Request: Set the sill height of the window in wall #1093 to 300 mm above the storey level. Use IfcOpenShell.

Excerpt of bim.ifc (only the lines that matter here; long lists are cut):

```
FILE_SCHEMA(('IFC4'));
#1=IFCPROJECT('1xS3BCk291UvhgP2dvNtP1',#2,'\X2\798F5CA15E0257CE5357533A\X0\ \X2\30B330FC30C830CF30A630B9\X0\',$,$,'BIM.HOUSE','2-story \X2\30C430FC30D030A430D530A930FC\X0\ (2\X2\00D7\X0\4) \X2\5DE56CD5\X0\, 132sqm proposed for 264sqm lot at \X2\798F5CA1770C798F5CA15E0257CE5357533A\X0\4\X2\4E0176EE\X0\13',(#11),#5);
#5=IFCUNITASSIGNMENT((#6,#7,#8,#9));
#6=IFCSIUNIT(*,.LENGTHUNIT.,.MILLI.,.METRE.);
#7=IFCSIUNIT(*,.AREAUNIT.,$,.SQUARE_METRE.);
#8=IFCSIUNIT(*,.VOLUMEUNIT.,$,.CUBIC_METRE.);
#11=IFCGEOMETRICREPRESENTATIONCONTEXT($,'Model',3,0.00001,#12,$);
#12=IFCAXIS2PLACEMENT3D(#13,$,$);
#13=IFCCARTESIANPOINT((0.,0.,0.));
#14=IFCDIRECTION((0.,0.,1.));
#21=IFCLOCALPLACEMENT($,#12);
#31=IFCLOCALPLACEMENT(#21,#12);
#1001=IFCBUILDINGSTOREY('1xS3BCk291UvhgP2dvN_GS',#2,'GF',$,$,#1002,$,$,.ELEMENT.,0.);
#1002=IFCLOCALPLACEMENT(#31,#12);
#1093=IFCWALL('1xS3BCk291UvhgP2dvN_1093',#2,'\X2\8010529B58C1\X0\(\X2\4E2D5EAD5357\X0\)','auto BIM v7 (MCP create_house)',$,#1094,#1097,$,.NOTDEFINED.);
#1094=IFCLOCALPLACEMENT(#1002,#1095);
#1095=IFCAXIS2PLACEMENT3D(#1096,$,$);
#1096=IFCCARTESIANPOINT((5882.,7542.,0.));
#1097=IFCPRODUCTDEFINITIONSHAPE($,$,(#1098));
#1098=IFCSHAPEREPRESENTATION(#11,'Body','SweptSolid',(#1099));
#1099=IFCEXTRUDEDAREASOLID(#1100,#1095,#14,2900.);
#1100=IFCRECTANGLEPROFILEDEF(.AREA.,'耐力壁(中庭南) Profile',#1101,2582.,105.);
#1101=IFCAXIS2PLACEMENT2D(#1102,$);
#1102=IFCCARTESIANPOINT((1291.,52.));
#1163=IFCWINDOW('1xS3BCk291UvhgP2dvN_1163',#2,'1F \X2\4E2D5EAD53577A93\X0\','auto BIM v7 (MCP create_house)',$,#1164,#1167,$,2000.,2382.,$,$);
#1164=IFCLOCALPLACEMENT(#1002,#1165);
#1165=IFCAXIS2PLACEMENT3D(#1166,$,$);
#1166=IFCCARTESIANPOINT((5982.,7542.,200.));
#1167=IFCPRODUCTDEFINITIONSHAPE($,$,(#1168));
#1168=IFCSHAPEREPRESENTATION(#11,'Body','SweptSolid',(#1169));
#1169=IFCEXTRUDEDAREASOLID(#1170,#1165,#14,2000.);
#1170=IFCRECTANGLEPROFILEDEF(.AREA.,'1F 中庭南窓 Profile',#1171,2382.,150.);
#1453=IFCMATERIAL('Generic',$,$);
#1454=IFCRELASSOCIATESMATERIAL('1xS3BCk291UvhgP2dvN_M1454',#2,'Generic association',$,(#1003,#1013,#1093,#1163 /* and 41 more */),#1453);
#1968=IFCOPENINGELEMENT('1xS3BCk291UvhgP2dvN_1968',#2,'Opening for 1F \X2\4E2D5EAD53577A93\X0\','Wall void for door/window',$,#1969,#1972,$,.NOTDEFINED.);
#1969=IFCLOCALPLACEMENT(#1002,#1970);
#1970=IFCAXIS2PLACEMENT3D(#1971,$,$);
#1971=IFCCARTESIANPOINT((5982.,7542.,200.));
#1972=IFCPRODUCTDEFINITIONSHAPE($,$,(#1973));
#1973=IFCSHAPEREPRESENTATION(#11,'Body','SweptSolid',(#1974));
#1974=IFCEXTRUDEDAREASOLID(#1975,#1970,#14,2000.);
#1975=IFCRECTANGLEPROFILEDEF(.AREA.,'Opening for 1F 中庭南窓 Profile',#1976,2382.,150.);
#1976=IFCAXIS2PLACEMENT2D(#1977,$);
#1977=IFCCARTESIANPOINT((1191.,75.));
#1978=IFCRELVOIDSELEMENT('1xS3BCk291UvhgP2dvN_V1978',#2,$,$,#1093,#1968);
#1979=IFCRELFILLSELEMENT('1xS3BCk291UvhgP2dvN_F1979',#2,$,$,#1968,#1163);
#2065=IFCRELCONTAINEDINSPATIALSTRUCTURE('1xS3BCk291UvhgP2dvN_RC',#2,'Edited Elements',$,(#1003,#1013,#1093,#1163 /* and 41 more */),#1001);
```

```python
import numpy as np
import ifcopenshell
import ifcopenshell.api.geometry
import ifcopenshell.geom
import ifcopenshell.util.element
import ifcopenshell.util.placement
import ifcopenshell.util.shape
import ifcopenshell.util.unit

model = ifcopenshell.open("bim.ifc")
unit_scale = ifcopenshell.util.unit.calculate_unit_scale(model)

window = model.by_guid("1xS3BCk291UvhgP2dvN_1163")
opening = window.FillsVoids[0].RelatingOpeningElement
storey = ifcopenshell.util.element.get_container(window, ifc_class="IfcBuildingStorey")
level = ifcopenshell.util.placement.get_local_placement(storey.ObjectPlacement)[2, 3]

# The opening's origin need not be at the sill, so measure its lowest point.
shape = ifcopenshell.geom.create_shape(ifcopenshell.geom.settings(), opening)
bottom = ifcopenshell.util.shape.get_shape_bottom_elevation(shape, shape.geometry) / unit_scale
dz = level + 300.0 - bottom

shift = np.array([0.0, 0.0, dz])
# The window is not placed relative to its opening, so move both.
for product in (opening, window):
    matrix = ifcopenshell.util.placement.get_local_placement(product.ObjectPlacement)
    matrix[:3, 3] += shift
    ifcopenshell.api.geometry.edit_object_placement(model, product=product, matrix=matrix, is_si=False)

print(f"moved by {dz * unit_scale:+.3f} m")

model.write("bim-out.ifc")
```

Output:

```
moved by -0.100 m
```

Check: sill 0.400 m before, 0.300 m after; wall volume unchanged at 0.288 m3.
